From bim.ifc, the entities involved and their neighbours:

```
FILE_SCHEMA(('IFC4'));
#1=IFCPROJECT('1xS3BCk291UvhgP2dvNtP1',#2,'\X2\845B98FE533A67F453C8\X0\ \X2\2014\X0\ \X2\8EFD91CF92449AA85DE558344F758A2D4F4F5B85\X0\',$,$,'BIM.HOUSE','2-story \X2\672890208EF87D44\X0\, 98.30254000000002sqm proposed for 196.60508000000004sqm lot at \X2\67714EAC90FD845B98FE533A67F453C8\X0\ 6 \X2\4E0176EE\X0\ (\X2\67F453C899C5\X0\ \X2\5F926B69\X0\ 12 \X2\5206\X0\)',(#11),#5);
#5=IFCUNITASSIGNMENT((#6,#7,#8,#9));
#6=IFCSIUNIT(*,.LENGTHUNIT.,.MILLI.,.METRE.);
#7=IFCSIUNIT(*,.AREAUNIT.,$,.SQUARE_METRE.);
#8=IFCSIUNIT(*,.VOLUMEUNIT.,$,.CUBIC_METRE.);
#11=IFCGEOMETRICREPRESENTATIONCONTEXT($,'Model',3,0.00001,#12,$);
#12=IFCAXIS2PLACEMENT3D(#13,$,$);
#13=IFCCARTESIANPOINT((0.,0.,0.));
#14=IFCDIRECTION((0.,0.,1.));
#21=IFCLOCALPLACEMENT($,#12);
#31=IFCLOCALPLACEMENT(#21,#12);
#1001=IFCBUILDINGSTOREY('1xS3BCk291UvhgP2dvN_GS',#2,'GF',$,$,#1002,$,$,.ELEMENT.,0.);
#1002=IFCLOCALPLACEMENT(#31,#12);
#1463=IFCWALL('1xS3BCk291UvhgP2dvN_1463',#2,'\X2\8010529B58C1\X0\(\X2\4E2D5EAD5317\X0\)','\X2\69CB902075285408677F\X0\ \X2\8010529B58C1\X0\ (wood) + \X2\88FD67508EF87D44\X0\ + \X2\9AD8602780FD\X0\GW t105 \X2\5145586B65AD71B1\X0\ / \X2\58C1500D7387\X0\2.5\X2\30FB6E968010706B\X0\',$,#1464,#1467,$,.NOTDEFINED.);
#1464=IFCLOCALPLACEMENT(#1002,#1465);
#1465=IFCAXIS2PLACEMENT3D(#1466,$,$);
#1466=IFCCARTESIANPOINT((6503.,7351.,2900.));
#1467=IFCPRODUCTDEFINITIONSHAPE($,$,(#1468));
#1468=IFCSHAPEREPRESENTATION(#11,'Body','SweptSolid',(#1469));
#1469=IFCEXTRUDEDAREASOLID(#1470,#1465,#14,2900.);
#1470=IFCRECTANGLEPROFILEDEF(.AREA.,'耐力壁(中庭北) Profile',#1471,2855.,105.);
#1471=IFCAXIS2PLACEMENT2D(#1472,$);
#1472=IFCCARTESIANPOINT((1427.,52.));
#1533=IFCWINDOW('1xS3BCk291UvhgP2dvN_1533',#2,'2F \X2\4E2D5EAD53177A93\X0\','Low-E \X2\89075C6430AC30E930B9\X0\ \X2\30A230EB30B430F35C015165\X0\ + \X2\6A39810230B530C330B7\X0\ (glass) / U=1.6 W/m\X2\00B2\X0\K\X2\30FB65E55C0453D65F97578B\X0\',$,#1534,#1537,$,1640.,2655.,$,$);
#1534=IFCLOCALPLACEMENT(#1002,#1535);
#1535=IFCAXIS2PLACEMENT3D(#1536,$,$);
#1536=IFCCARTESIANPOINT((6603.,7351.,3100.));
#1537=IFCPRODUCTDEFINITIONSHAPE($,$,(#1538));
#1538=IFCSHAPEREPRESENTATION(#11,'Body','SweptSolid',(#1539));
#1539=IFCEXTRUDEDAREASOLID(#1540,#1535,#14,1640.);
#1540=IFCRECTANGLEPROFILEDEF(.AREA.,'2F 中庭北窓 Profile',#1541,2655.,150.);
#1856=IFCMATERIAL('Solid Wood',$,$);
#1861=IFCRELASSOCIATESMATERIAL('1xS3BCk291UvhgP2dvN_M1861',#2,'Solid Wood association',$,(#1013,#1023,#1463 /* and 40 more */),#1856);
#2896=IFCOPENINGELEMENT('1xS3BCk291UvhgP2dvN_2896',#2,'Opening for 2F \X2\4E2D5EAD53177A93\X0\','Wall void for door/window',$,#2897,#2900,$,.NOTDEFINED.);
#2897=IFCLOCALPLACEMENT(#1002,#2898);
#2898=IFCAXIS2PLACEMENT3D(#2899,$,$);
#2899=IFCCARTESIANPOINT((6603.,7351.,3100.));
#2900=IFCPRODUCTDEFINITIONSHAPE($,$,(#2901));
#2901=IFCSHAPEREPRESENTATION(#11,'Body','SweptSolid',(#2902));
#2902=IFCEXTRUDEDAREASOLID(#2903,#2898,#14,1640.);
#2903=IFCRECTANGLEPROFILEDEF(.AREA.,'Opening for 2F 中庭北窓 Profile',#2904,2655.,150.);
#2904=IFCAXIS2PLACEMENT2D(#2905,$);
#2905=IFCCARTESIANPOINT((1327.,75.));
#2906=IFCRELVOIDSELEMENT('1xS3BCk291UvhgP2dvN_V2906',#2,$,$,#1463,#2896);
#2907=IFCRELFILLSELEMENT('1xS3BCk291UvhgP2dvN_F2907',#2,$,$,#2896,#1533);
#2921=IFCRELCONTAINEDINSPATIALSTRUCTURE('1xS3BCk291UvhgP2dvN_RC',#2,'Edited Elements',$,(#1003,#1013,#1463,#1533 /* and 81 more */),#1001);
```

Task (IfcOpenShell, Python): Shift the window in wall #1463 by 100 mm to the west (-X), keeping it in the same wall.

```python
import ifcopenshell
import ifcopenshell.api.geometry
import ifcopenshell.util.placement
import ifcopenshell.util.unit

model = ifcopenshell.open("bim.ifc")
unit_scale = ifcopenshell.util.unit.calculate_unit_scale(model)

window = model.by_guid("1xS3BCk291UvhgP2dvN_1533")
opening = window.FillsVoids[0].RelatingOpeningElement
wall = opening.VoidsElements[0].RelatingBuildingElement

wall_matrix = ifcopenshell.util.placement.get_local_placement(wall.ObjectPlacement)
shift = wall_matrix[:3, 0] * -0.1 / unit_scale
before = ifcopenshell.util.placement.get_local_placement(window.ObjectPlacement)[:3, 3].copy()

# The window is not placed relative to its opening, so move both.
for product in (opening, window):
    matrix = ifcopenshell.util.placement.get_local_placement(product.ObjectPlacement)
    matrix[:3, 3] += shift
    ifcopenshell.api.geometry.edit_object_placement(model, product=product, matrix=matrix, is_si=False)

after = ifcopenshell.util.placement.get_local_placement(window.ObjectPlacement)[:3, 3]
print("window moved by", (after - before).round(3) + 0.0)

model.write("bim-out.ifc")
```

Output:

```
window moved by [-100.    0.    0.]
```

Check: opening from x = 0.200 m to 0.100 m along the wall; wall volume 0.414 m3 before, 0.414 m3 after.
